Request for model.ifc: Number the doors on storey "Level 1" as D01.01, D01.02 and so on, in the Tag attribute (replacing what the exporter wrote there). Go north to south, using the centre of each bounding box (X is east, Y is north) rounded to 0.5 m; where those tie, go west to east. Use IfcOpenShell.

First a look at what the model holds.

```python
import ifcopenshell
import ifcopenshell.util.element
import ifcopenshell.util.placement

model = ifcopenshell.open("model.ifc")
print(model.schema)
storey = next(s for s in model.by_type("IfcBuildingStorey") if s.Name == "Level 1")
doors = [e for e in ifcopenshell.util.element.get_decomposition(storey) if e.is_a("IfcDoor")]
for e in sorted(doors, key=lambda e: e.id()):
    origin = ifcopenshell.util.placement.get_local_placement(e.ObjectPlacement)[:3, 3]
    print(e.id(), e.Tag, e.Name, origin.round(2) + 0.0, sep=" | ")
```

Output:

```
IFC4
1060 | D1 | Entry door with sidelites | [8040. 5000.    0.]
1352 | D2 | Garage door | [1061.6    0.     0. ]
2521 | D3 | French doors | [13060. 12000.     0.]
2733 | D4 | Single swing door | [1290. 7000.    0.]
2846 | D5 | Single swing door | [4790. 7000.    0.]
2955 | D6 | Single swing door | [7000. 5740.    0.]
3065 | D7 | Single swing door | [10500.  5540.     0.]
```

```python
import ifcopenshell
import ifcopenshell.geom
import ifcopenshell.util.element
import ifcopenshell.util.shape

model = ifcopenshell.open("model.ifc")
settings = ifcopenshell.geom.settings()
settings.set("use-world-coords", True)


def centre(element):
    shape = ifcopenshell.geom.create_shape(settings, element)
    return ifcopenshell.util.shape.get_bbox_centroid(shape.geometry)


storey = next(s for s in model.by_type("IfcBuildingStorey") if s.Name == "Level 1")
doors = [e for e in ifcopenshell.util.element.get_decomposition(storey) if e.is_a("IfcDoor")]

# Insertion points can sit at a corner or the storey origin, so sort by the geometry (in metres).
centres = {e: centre(e) for e in doors}
doors.sort(key=lambda e: (-round(centres[e][1] / 0.5), centres[e][0]))

for i, e in enumerate(doors, start=1):
    number = f"D01.{i:02d}"
    e.Tag = number
    print(e.id(), number)

model.write("model_updated.ifc")
```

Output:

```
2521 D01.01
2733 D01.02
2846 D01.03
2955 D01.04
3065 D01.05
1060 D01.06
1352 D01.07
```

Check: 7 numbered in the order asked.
